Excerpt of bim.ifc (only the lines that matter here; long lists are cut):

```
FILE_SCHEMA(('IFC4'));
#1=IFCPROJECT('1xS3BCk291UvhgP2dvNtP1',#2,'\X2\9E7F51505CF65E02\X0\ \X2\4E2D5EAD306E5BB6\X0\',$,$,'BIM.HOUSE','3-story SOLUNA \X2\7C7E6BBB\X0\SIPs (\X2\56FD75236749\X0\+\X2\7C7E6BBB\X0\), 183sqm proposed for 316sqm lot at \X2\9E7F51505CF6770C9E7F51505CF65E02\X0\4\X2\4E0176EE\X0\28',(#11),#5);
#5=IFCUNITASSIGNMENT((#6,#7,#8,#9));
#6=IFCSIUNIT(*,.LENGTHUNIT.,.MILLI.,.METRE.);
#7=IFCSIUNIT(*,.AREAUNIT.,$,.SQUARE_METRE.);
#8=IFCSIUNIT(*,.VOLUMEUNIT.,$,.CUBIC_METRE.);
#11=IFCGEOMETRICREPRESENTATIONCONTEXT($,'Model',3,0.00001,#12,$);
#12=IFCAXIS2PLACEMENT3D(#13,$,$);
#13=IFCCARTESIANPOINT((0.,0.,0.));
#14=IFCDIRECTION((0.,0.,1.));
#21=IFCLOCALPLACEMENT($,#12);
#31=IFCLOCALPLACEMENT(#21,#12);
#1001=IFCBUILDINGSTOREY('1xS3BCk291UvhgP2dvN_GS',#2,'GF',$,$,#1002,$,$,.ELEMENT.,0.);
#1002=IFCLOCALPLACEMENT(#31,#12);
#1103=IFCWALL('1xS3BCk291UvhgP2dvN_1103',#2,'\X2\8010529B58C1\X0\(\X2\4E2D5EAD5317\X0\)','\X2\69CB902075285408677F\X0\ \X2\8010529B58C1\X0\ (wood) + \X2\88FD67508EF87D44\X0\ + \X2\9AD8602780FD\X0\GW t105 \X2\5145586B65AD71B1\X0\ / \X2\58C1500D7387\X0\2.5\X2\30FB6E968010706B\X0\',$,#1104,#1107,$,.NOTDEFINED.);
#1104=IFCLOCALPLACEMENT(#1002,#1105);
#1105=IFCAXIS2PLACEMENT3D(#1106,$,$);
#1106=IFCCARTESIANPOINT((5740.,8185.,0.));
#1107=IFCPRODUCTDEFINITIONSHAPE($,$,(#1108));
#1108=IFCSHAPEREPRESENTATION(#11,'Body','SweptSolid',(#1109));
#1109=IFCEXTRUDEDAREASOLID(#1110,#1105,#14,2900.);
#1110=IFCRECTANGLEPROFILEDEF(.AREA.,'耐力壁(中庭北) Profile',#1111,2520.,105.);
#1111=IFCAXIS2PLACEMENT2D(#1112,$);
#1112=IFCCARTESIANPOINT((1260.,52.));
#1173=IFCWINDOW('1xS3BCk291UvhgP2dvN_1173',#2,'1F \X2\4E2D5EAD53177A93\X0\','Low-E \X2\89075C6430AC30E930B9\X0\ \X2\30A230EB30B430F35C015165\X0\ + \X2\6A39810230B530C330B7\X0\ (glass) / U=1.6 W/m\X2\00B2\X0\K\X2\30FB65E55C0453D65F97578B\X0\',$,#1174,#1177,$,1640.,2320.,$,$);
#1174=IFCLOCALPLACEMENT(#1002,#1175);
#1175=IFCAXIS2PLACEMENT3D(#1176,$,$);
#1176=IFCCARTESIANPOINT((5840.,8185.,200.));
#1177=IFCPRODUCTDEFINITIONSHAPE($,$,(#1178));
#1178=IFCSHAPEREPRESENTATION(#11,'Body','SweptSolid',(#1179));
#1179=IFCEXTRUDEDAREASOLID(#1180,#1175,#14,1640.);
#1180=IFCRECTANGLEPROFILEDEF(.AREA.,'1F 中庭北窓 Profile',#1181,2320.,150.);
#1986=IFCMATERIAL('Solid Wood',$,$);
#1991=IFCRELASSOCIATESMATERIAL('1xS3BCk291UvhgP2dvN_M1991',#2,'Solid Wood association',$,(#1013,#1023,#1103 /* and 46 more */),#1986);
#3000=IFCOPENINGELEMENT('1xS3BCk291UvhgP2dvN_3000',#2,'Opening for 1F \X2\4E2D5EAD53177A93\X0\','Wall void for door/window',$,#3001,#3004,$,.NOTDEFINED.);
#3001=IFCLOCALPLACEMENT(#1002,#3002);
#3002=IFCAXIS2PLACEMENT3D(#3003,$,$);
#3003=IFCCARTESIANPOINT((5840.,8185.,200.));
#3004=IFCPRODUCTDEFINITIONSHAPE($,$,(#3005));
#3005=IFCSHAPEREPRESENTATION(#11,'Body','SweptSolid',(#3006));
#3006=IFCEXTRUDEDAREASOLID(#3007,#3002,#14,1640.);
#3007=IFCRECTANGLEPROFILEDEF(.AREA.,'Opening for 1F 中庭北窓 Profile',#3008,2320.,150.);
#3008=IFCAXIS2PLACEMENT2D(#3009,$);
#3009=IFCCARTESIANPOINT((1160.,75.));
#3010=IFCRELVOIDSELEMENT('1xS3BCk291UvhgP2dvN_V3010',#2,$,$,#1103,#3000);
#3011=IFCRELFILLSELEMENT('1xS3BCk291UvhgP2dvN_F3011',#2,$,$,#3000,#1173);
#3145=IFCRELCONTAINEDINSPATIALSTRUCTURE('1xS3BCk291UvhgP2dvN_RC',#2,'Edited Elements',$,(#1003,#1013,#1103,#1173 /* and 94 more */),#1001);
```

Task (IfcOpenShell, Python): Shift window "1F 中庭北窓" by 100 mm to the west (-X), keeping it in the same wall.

```python
import ifcopenshell
import ifcopenshell.api.geometry
import ifcopenshell.util.placement
import ifcopenshell.util.unit

model = ifcopenshell.open("bim.ifc")
unit_scale = ifcopenshell.util.unit.calculate_unit_scale(model)

window = model.by_guid("1xS3BCk291UvhgP2dvN_1173")
opening = window.FillsVoids[0].RelatingOpeningElement
wall = opening.VoidsElements[0].RelatingBuildingElement

wall_matrix = ifcopenshell.util.placement.get_local_placement(wall.ObjectPlacement)
shift = wall_matrix[:3, 0] * -0.1 / unit_scale
before = ifcopenshell.util.placement.get_local_placement(window.ObjectPlacement)[:3, 3].copy()

# The window is not placed relative to its opening, so move both.
for product in (opening, window):
    matrix = ifcopenshell.util.placement.get_local_placement(product.ObjectPlacement)
    matrix[:3, 3] += shift
    ifcopenshell.api.geometry.edit_object_placement(model, product=product, matrix=matrix, is_si=False)

after = ifcopenshell.util.placement.get_local_placement(window.ObjectPlacement)[:3, 3]
print("window moved by", (after - before).round(3) + 0.0)

model.write("bim_edited.ifc")
```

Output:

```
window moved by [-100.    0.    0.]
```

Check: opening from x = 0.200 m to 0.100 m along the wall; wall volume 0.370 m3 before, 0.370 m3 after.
